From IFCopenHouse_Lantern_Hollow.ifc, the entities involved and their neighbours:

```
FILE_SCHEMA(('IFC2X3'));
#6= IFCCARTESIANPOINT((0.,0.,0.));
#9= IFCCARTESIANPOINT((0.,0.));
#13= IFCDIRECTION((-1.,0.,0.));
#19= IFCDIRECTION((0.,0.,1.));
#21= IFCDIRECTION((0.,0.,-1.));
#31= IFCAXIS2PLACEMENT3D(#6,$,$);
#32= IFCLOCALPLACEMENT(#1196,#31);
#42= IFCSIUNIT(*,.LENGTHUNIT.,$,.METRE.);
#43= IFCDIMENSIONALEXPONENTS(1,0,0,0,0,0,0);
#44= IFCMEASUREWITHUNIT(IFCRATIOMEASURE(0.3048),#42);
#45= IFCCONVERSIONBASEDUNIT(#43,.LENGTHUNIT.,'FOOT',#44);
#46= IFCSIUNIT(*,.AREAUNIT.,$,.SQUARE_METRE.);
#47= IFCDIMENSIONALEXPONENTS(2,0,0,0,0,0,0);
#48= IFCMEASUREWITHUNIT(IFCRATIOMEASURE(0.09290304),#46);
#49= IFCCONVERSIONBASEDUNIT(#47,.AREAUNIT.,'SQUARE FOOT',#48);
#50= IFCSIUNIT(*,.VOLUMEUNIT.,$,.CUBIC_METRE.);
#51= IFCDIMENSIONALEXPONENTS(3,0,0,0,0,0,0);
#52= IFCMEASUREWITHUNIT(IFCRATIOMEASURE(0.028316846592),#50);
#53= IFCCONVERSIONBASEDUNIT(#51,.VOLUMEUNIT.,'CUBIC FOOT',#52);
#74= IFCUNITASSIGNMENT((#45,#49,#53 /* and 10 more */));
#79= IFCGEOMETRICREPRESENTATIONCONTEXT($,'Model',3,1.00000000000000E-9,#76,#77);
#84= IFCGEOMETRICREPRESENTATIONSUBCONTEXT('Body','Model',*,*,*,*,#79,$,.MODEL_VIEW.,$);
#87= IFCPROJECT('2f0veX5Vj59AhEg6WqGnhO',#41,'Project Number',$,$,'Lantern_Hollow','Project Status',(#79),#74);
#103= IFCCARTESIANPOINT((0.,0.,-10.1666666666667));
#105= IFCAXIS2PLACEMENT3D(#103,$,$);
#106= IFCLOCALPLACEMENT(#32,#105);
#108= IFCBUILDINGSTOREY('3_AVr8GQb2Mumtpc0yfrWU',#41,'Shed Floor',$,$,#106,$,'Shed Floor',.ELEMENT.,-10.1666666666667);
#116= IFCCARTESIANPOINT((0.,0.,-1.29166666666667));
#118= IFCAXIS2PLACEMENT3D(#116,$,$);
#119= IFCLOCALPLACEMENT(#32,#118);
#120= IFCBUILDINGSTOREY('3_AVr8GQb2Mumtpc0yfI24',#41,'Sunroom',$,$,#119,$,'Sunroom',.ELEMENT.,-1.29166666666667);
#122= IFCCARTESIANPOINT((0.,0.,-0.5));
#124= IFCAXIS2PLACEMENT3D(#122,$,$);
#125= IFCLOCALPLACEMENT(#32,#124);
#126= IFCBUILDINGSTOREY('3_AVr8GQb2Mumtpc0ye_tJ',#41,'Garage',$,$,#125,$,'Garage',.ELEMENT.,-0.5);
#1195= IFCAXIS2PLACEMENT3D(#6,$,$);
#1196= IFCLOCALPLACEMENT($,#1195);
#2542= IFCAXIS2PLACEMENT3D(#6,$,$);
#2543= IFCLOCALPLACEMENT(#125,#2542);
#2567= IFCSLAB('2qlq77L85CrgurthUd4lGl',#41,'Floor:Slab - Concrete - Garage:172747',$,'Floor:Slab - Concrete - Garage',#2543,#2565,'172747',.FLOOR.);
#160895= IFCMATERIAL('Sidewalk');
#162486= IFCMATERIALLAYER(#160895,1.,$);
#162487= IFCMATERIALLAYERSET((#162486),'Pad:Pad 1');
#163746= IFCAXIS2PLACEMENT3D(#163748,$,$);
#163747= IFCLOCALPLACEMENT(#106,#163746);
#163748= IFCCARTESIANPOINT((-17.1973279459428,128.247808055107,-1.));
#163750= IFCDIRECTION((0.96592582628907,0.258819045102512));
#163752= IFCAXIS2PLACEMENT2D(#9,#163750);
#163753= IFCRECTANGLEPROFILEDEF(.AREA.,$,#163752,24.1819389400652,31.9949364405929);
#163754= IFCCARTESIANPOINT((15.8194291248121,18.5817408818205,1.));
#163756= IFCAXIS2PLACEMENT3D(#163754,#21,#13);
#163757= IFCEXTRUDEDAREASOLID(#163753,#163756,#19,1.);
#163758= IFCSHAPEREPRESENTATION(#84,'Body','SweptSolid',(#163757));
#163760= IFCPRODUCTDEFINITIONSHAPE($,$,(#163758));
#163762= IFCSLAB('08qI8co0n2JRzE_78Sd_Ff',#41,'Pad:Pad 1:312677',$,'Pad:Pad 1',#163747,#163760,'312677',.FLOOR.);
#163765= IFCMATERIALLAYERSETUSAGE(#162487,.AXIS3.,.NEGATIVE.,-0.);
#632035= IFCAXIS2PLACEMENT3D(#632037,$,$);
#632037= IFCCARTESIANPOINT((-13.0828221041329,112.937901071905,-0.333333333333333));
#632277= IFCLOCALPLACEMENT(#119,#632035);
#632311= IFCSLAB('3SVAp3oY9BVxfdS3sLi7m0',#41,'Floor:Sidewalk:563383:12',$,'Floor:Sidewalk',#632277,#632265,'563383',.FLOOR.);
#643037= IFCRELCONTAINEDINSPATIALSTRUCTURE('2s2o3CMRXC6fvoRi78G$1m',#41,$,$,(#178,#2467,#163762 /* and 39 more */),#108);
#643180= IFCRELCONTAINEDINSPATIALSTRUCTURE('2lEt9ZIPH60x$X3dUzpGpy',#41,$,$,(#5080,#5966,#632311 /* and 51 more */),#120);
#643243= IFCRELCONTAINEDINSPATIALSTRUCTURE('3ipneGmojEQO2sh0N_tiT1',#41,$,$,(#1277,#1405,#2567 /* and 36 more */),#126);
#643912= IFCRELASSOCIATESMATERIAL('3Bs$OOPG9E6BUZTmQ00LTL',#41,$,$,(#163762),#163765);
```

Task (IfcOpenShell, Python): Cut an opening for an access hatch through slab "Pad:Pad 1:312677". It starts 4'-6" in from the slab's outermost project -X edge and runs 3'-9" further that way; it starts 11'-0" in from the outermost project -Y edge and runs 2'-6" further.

```python
import numpy as np
import ifcopenshell
import ifcopenshell.api.feature
import ifcopenshell.api.geometry
import ifcopenshell.api.root
import ifcopenshell.geom
import ifcopenshell.util.placement
import ifcopenshell.util.representation
import ifcopenshell.util.shape
import ifcopenshell.util.unit

model = ifcopenshell.open("IFCopenHouse_Lantern_Hollow.ifc")
unit_scale = ifcopenshell.util.unit.calculate_unit_scale(model)
settings = ifcopenshell.geom.settings()


def volume(element):
    """Net volume in cubic metres, openings subtracted."""
    shape = ifcopenshell.geom.create_shape(settings, element)
    return ifcopenshell.util.shape.get_volume(shape.geometry)


slab = model.by_guid("08qI8co0n2JRzE_78Sd_Ff")
before = volume(slab)

# Extent in the slab's own axes, in metres. The edges named are its -X and -Y sides.
slab_shape = ifcopenshell.geom.create_shape(settings, slab)
vertices = ifcopenshell.util.shape.get_vertices(slab_shape.geometry)
x_min, y_min, bottom = vertices.min(axis=0)
top = vertices[:, 2].max()

opening = ifcopenshell.api.root.create_entity(model, ifc_class="IfcOpeningElement", name="Access hatch opening")
context = ifcopenshell.util.representation.get_context(model, "Model", "Body", "MODEL_VIEW")
width, depth = 1.143, 0.762
outline = [(0.0, 0.0), (width, 0.0), (width, depth), (0.0, depth), (0.0, 0.0)]
# Overshoot both faces by 50 mm so the cut is clean.
shape = ifcopenshell.api.geometry.add_slab_representation(
    model, context=context, depth=top - bottom + 0.1, polyline=outline
)
ifcopenshell.api.geometry.assign_representation(model, product=opening, representation=shape)

matrix = ifcopenshell.util.placement.get_local_placement(slab.ObjectPlacement)
matrix[:, 3] = matrix @ np.append(np.array([x_min + 1.3716, y_min + 3.3528, bottom - 0.05]) / unit_scale, 1.0)
ifcopenshell.api.geometry.edit_object_placement(model, product=opening, matrix=matrix, is_si=False)
ifcopenshell.api.feature.add_feature(model, feature=opening, element=slab)

after = volume(slab)

print(f"slab volume {before:.3f} -> {after:.3f} m3")

model.write("IFCopenHouse_Lantern_Hollow-out.ifc")
```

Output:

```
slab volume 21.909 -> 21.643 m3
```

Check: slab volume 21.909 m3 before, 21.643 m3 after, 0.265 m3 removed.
